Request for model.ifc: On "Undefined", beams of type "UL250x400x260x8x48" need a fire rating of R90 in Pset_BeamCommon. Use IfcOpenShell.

First a look at what the model holds.

```python
import ifcopenshell
import ifcopenshell.util.element

model = ifcopenshell.open("model.ifc")
print(model.schema)
storey = next(s for s in model.by_type("IfcBuildingStorey") if s.Name == "Undefined")
beams = [e for e in ifcopenshell.util.element.get_decomposition(storey) if e.is_a("IfcBeam")]
seen = {}
for e in beams:
    element_type = ifcopenshell.util.element.get_type(e)
    key = (element_type.Name if element_type != e and element_type else None, ifcopenshell.util.element.get_pset(e, "Pset_BeamCommon", "FireRating"))
    seen[key] = seen.get(key, 0) + 1
for (name, value), count in sorted(seen.items(), key=str):
    print(count, "x", name, "|", value)
```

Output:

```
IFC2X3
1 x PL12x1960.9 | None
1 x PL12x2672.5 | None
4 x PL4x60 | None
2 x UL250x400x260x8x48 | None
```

```python
import ifcopenshell
import ifcopenshell.api.pset
import ifcopenshell.util.element

model = ifcopenshell.open("model.ifc")

storey = next(s for s in model.by_type("IfcBuildingStorey") if s.Name == "Undefined")
beams = [e for e in ifcopenshell.util.element.get_decomposition(storey) if e.is_a("IfcBeam")]

count = 0
for e in beams:
    element_type = ifcopenshell.util.element.get_type(e)
    if element_type in (None, e) or element_type.Name != "UL250x400x260x8x48":
        continue
    # add_pset returns the element's existing set when there is one.
    pset = ifcopenshell.api.pset.add_pset(model, product=e, name="Pset_BeamCommon")
    ifcopenshell.api.pset.edit_pset(model, pset=pset, properties={"FireRating": "R90"})
    count += 1

print(count, "beams updated")

model.write("model-out.ifc")
```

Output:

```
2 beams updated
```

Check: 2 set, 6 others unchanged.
